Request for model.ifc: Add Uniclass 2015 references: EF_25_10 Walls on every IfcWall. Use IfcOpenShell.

First a look at what the model holds.

```python
import ifcopenshell

model = ifcopenshell.open("model.ifc")
print(model.schema)
print("classifications:", [c.Name for c in model.by_type("IfcClassification")])
for ifc_class in ("IfcDoor", "IfcRoof", "IfcStair", "IfcWall", "IfcWindow"):
    print(ifc_class, len(model.by_type(ifc_class)))
```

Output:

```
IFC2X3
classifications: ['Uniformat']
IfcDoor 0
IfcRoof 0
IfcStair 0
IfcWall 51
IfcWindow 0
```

```python
import ifcopenshell
import ifcopenshell.api.classification

model = ifcopenshell.open("model.ifc")

# IFC2X3 requires Source and Edition and has no link from the project to the system.
system = model.create_entity("IfcClassification", Source="NBS", Edition="2015", Name="Uniclass 2015")

codes = {
    "IfcWall": ("EF_25_10", "Walls"),
}
for ifc_class, (code, name) in codes.items():
    products = model.by_type(ifc_class)
    ifcopenshell.api.classification.add_reference(
        model, products=products, classification=system, identification=code, name=name
    )
    print(code, len(products))

model.write("model_v2.ifc")
```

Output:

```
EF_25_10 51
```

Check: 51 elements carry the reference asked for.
